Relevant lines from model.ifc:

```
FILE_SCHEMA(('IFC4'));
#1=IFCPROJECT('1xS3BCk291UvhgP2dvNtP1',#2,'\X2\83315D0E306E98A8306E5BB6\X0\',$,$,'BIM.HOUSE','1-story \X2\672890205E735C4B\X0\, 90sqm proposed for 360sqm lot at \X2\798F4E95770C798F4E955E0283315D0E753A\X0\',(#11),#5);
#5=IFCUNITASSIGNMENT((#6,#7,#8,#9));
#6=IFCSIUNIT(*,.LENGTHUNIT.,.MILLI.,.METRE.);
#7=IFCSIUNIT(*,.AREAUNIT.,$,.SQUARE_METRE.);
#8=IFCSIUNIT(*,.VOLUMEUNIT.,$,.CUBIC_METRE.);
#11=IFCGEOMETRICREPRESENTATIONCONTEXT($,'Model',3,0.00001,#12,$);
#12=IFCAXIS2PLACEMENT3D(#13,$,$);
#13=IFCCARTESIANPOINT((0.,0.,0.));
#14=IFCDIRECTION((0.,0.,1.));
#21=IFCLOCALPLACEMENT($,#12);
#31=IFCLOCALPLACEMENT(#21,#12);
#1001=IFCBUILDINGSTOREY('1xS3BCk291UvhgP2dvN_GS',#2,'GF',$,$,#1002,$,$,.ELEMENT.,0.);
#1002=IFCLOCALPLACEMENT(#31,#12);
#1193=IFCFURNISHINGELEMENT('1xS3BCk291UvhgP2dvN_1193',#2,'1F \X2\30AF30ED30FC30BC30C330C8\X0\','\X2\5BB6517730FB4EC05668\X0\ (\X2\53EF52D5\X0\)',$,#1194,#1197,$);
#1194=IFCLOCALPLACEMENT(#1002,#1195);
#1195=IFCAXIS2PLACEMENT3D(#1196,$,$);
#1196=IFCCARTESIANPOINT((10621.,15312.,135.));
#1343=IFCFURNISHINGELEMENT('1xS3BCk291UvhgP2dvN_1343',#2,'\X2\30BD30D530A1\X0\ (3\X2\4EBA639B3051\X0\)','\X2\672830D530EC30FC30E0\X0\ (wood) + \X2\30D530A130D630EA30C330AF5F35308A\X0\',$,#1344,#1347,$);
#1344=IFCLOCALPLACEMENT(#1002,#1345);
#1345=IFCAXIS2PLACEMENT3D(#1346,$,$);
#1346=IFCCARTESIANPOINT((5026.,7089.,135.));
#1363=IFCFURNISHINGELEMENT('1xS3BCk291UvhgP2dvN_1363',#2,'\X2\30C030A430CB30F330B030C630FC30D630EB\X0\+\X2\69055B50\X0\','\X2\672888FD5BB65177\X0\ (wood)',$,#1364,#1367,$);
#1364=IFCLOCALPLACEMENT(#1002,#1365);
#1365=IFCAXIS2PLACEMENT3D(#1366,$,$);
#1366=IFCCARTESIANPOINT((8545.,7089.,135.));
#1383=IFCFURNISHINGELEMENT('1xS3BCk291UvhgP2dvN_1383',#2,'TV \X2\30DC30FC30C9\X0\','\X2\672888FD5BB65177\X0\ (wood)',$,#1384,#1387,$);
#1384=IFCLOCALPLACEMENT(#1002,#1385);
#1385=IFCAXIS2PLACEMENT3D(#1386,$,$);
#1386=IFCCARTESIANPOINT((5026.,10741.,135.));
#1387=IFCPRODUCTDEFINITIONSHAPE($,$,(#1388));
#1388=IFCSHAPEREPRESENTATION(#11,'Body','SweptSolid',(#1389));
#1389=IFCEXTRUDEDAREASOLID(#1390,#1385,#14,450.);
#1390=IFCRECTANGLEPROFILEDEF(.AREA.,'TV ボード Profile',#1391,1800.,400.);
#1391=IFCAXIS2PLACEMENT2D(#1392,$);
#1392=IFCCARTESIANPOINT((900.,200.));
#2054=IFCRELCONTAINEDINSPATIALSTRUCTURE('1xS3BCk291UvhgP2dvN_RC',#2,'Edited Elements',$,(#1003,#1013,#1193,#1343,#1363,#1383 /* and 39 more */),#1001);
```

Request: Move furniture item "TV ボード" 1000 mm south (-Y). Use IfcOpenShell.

```python
import ifcopenshell
import ifcopenshell.api.geometry
import ifcopenshell.util.placement

model = ifcopenshell.open("model.ifc")

item = model.by_id(1383)
matrix = ifcopenshell.util.placement.get_local_placement(item.ObjectPlacement)
matrix[1, 3] -= 1000.0
ifcopenshell.api.geometry.edit_object_placement(model, product=item, matrix=matrix, is_si=False)

print(ifcopenshell.util.placement.get_local_placement(item.ObjectPlacement).round(3) + 0.0)

model.write("model-out.ifc")
```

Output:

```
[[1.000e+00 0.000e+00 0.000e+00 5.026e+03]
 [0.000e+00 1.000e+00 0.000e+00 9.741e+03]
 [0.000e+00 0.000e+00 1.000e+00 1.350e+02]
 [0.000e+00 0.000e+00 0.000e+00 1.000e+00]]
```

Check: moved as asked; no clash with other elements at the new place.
